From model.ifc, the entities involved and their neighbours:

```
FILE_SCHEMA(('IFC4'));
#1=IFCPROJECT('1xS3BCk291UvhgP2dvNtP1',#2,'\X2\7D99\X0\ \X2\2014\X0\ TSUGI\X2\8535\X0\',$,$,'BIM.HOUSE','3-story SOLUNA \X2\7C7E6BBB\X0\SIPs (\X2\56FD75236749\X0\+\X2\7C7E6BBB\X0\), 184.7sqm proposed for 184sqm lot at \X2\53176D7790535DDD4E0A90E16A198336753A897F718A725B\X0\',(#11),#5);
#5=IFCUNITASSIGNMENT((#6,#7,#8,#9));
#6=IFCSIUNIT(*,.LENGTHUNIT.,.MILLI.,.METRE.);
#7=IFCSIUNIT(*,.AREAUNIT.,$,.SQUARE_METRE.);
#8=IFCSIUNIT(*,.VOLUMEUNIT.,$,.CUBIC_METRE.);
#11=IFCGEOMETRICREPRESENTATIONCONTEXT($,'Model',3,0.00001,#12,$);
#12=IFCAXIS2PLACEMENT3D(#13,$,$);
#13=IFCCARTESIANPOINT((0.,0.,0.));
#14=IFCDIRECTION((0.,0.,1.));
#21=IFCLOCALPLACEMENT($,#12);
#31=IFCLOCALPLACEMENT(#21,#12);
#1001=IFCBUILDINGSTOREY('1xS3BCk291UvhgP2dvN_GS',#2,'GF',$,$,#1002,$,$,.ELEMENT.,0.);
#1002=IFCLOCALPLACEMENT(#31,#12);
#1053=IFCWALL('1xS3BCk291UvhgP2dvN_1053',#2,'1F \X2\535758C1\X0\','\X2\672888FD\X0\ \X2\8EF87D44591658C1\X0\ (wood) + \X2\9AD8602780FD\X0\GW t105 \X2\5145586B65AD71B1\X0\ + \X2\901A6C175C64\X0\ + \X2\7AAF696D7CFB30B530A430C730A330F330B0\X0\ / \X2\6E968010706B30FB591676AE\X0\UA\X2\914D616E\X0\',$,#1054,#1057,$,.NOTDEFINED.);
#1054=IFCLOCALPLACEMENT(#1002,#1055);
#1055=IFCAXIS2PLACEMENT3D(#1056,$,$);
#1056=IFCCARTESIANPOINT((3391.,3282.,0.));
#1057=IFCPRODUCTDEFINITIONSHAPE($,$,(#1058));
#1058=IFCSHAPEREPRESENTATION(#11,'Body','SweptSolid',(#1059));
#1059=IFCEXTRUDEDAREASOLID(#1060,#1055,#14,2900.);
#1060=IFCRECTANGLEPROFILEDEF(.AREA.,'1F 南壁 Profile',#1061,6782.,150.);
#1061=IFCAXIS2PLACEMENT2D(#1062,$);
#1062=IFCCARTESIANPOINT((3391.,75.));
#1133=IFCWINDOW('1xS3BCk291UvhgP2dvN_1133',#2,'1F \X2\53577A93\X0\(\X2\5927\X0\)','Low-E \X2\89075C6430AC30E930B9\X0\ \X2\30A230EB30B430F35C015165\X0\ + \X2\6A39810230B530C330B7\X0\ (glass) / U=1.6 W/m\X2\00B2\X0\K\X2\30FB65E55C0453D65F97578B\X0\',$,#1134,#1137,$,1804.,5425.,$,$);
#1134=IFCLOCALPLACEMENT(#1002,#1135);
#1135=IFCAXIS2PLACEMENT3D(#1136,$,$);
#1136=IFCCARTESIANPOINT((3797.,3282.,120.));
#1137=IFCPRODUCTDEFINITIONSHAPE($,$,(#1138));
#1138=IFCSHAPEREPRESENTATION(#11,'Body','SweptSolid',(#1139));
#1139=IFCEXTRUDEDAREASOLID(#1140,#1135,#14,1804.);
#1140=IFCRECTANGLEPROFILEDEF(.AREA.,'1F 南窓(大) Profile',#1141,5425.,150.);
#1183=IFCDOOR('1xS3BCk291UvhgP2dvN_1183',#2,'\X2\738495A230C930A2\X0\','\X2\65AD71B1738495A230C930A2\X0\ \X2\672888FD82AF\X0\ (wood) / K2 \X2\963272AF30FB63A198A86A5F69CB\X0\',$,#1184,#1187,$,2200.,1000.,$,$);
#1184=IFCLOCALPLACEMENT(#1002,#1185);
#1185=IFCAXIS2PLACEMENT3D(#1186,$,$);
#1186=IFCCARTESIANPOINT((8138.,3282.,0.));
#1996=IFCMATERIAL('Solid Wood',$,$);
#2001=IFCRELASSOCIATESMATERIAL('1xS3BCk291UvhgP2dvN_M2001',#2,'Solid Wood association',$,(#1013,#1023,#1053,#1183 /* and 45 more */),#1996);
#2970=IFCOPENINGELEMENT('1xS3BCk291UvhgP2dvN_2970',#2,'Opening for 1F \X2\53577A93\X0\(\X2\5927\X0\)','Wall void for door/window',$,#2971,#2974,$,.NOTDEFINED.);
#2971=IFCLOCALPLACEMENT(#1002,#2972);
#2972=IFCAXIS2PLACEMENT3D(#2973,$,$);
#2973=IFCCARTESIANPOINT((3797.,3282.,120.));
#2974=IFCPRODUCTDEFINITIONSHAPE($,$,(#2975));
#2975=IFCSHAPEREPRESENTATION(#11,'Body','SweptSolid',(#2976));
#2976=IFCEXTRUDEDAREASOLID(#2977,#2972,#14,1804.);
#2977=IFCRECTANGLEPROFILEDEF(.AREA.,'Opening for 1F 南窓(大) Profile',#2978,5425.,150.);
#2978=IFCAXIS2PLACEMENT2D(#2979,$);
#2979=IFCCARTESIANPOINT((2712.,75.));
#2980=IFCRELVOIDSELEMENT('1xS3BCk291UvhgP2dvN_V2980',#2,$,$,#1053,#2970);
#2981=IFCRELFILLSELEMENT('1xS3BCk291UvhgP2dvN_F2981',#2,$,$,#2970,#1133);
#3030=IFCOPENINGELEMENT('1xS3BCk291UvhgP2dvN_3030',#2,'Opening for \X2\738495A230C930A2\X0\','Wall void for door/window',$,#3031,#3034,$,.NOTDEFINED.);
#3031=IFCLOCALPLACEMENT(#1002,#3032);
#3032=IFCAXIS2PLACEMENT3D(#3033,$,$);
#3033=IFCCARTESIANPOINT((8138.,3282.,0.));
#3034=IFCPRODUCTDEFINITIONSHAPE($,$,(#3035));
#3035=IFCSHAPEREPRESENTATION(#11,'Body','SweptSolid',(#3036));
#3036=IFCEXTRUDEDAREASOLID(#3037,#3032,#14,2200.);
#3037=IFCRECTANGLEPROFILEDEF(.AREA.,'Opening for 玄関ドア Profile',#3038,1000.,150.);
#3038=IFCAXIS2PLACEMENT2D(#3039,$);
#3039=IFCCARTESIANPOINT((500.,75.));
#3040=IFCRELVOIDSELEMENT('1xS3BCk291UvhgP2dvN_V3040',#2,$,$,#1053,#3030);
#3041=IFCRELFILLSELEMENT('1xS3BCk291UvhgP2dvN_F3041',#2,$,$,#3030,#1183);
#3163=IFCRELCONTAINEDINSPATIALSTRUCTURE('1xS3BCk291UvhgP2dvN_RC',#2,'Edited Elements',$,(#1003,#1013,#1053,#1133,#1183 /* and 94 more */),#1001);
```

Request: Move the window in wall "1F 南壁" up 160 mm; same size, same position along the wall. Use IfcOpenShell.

```python
import numpy as np
import ifcopenshell
import ifcopenshell.api.geometry
import ifcopenshell.util.placement
import ifcopenshell.util.unit

model = ifcopenshell.open("model.ifc")
unit_scale = ifcopenshell.util.unit.calculate_unit_scale(model)

window = model.by_guid("1xS3BCk291UvhgP2dvN_1133")
opening = window.FillsVoids[0].RelatingOpeningElement
dz = 0.16 / unit_scale

shift = np.array([0.0, 0.0, dz])
# The window is not placed relative to its opening, so move both.
for product in (opening, window):
    matrix = ifcopenshell.util.placement.get_local_placement(product.ObjectPlacement)
    matrix[:3, 3] += shift
    ifcopenshell.api.geometry.edit_object_placement(model, product=product, matrix=matrix, is_si=False)

print(f"moved by {dz * unit_scale:+.3f} m")

model.write("model-out.ifc")
```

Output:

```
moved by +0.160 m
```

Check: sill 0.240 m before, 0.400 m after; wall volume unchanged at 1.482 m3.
